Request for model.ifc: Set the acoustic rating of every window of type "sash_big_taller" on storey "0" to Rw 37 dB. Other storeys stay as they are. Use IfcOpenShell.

First a look at what the model holds.

```python
import ifcopenshell
import ifcopenshell.util.element

model = ifcopenshell.open("model.ifc")
print(model.schema)
storey = next(s for s in model.by_type("IfcBuildingStorey") if s.Name == "0")
windows = [e for e in ifcopenshell.util.element.get_decomposition(storey) if e.is_a("IfcWindow")]
seen = {}
for e in windows:
    element_type = ifcopenshell.util.element.get_type(e)
    key = (element_type.Name if element_type != e and element_type else None, ifcopenshell.util.element.get_pset(e, "Pset_WindowCommon", "AcousticRating"))
    seen[key] = seen.get(key, 0) + 1
for (name, value), count in sorted(seen.items(), key=str):
    print(count, "x", name, "|", value)
```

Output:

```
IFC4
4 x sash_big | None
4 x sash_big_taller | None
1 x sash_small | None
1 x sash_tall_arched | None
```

```python
import ifcopenshell
import ifcopenshell.api.pset
import ifcopenshell.util.element

model = ifcopenshell.open("model.ifc")

storey = next(s for s in model.by_type("IfcBuildingStorey") if s.Name == "0")
windows = [e for e in ifcopenshell.util.element.get_decomposition(storey) if e.is_a("IfcWindow")]

count = 0
for e in windows:
    element_type = ifcopenshell.util.element.get_type(e)
    if element_type in (None, e) or element_type.Name != "sash_big_taller":
        continue
    # add_pset returns the element's existing set when there is one.
    pset = ifcopenshell.api.pset.add_pset(model, product=e, name="Pset_WindowCommon")
    ifcopenshell.api.pset.edit_pset(model, pset=pset, properties={"AcousticRating": "Rw 37 dB"})
    count += 1

print(count, "windows updated")

model.write("model_updated.ifc")
```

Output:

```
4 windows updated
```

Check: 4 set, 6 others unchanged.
